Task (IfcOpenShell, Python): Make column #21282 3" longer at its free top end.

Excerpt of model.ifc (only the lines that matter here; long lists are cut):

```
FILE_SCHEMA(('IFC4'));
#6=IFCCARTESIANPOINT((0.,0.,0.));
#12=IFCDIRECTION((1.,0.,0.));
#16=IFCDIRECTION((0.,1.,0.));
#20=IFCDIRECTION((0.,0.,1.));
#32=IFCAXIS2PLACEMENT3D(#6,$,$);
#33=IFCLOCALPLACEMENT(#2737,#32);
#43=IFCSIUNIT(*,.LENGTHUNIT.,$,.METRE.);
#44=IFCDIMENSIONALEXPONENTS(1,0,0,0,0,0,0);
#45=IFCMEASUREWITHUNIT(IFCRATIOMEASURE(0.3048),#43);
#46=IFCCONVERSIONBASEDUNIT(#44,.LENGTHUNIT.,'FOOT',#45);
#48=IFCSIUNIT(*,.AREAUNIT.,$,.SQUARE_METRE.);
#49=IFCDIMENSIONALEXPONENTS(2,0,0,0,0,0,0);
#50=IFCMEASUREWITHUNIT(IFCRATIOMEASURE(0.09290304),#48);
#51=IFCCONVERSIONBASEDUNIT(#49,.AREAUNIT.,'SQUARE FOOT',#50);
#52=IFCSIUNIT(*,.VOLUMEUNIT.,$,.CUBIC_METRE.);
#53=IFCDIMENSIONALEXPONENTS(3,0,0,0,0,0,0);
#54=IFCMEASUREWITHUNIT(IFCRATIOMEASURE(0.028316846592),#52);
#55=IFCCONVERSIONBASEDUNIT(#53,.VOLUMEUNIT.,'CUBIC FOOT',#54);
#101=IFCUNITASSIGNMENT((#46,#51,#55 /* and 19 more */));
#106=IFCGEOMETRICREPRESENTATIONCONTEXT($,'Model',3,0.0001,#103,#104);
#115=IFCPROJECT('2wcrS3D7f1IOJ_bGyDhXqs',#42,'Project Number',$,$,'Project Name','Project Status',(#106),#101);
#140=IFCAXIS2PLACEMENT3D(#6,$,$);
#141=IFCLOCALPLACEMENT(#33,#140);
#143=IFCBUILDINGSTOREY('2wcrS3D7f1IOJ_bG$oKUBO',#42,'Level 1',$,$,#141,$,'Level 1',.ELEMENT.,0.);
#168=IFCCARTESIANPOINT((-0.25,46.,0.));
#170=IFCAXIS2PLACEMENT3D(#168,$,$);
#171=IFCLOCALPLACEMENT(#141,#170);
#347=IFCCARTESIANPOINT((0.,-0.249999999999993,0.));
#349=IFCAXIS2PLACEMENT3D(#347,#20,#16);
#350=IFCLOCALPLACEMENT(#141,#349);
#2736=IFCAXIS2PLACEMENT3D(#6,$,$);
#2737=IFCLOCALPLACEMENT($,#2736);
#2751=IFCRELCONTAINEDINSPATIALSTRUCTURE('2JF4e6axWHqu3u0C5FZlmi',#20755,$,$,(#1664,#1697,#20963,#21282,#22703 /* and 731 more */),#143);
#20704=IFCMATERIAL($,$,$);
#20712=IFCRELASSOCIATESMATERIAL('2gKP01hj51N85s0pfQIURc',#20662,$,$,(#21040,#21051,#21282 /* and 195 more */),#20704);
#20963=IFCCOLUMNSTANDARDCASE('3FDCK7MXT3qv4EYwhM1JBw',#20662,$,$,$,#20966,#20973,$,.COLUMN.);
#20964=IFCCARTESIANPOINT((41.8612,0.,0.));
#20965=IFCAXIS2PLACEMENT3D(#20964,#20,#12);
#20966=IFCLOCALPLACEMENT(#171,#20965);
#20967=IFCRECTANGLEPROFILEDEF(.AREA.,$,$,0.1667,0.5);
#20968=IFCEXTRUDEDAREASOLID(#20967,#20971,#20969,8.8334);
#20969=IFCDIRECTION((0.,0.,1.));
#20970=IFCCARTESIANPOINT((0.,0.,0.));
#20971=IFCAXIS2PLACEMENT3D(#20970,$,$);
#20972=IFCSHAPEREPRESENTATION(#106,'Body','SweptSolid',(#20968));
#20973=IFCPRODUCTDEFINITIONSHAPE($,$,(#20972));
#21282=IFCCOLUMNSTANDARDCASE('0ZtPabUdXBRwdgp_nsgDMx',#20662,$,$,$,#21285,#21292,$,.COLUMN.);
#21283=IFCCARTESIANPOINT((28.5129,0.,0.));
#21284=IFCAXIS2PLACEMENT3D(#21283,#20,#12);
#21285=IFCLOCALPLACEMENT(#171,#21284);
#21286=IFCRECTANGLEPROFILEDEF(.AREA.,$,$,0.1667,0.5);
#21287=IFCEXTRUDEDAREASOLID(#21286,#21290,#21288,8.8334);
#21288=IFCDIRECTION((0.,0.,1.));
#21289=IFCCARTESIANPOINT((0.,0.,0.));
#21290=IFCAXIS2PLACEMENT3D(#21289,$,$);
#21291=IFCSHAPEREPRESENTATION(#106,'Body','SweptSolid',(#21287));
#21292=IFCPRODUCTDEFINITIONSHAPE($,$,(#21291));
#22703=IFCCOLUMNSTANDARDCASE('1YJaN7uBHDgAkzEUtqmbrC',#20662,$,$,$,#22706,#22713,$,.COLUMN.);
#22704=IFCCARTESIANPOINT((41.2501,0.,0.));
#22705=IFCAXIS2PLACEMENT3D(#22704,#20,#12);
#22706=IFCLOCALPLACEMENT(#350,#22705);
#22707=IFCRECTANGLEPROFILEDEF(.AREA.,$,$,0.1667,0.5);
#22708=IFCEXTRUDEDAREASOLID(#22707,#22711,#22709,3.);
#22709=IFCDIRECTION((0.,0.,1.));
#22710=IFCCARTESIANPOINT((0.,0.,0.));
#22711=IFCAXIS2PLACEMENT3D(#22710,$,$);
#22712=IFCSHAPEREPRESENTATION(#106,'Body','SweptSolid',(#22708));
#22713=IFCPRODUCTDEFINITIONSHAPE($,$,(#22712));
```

```python
import ifcopenshell
import ifcopenshell.util.unit

model = ifcopenshell.open("model.ifc")
unit_scale = ifcopenshell.util.unit.calculate_unit_scale(model)

member = model.by_id(21282)
change = 3 * 0.0254 / unit_scale

# The extrusion runs towards the end named, so only its depth changes.
body = next(r for r in member.Representation.Representations if r.RepresentationIdentifier == "Body")
solid = body.Items[0]
old_length = solid.Depth
solid.Depth += change

print(f"length {old_length:g} -> {solid.Depth:g}")

model.write("model-out.ifc")
```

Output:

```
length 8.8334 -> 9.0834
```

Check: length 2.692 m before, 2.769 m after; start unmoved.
